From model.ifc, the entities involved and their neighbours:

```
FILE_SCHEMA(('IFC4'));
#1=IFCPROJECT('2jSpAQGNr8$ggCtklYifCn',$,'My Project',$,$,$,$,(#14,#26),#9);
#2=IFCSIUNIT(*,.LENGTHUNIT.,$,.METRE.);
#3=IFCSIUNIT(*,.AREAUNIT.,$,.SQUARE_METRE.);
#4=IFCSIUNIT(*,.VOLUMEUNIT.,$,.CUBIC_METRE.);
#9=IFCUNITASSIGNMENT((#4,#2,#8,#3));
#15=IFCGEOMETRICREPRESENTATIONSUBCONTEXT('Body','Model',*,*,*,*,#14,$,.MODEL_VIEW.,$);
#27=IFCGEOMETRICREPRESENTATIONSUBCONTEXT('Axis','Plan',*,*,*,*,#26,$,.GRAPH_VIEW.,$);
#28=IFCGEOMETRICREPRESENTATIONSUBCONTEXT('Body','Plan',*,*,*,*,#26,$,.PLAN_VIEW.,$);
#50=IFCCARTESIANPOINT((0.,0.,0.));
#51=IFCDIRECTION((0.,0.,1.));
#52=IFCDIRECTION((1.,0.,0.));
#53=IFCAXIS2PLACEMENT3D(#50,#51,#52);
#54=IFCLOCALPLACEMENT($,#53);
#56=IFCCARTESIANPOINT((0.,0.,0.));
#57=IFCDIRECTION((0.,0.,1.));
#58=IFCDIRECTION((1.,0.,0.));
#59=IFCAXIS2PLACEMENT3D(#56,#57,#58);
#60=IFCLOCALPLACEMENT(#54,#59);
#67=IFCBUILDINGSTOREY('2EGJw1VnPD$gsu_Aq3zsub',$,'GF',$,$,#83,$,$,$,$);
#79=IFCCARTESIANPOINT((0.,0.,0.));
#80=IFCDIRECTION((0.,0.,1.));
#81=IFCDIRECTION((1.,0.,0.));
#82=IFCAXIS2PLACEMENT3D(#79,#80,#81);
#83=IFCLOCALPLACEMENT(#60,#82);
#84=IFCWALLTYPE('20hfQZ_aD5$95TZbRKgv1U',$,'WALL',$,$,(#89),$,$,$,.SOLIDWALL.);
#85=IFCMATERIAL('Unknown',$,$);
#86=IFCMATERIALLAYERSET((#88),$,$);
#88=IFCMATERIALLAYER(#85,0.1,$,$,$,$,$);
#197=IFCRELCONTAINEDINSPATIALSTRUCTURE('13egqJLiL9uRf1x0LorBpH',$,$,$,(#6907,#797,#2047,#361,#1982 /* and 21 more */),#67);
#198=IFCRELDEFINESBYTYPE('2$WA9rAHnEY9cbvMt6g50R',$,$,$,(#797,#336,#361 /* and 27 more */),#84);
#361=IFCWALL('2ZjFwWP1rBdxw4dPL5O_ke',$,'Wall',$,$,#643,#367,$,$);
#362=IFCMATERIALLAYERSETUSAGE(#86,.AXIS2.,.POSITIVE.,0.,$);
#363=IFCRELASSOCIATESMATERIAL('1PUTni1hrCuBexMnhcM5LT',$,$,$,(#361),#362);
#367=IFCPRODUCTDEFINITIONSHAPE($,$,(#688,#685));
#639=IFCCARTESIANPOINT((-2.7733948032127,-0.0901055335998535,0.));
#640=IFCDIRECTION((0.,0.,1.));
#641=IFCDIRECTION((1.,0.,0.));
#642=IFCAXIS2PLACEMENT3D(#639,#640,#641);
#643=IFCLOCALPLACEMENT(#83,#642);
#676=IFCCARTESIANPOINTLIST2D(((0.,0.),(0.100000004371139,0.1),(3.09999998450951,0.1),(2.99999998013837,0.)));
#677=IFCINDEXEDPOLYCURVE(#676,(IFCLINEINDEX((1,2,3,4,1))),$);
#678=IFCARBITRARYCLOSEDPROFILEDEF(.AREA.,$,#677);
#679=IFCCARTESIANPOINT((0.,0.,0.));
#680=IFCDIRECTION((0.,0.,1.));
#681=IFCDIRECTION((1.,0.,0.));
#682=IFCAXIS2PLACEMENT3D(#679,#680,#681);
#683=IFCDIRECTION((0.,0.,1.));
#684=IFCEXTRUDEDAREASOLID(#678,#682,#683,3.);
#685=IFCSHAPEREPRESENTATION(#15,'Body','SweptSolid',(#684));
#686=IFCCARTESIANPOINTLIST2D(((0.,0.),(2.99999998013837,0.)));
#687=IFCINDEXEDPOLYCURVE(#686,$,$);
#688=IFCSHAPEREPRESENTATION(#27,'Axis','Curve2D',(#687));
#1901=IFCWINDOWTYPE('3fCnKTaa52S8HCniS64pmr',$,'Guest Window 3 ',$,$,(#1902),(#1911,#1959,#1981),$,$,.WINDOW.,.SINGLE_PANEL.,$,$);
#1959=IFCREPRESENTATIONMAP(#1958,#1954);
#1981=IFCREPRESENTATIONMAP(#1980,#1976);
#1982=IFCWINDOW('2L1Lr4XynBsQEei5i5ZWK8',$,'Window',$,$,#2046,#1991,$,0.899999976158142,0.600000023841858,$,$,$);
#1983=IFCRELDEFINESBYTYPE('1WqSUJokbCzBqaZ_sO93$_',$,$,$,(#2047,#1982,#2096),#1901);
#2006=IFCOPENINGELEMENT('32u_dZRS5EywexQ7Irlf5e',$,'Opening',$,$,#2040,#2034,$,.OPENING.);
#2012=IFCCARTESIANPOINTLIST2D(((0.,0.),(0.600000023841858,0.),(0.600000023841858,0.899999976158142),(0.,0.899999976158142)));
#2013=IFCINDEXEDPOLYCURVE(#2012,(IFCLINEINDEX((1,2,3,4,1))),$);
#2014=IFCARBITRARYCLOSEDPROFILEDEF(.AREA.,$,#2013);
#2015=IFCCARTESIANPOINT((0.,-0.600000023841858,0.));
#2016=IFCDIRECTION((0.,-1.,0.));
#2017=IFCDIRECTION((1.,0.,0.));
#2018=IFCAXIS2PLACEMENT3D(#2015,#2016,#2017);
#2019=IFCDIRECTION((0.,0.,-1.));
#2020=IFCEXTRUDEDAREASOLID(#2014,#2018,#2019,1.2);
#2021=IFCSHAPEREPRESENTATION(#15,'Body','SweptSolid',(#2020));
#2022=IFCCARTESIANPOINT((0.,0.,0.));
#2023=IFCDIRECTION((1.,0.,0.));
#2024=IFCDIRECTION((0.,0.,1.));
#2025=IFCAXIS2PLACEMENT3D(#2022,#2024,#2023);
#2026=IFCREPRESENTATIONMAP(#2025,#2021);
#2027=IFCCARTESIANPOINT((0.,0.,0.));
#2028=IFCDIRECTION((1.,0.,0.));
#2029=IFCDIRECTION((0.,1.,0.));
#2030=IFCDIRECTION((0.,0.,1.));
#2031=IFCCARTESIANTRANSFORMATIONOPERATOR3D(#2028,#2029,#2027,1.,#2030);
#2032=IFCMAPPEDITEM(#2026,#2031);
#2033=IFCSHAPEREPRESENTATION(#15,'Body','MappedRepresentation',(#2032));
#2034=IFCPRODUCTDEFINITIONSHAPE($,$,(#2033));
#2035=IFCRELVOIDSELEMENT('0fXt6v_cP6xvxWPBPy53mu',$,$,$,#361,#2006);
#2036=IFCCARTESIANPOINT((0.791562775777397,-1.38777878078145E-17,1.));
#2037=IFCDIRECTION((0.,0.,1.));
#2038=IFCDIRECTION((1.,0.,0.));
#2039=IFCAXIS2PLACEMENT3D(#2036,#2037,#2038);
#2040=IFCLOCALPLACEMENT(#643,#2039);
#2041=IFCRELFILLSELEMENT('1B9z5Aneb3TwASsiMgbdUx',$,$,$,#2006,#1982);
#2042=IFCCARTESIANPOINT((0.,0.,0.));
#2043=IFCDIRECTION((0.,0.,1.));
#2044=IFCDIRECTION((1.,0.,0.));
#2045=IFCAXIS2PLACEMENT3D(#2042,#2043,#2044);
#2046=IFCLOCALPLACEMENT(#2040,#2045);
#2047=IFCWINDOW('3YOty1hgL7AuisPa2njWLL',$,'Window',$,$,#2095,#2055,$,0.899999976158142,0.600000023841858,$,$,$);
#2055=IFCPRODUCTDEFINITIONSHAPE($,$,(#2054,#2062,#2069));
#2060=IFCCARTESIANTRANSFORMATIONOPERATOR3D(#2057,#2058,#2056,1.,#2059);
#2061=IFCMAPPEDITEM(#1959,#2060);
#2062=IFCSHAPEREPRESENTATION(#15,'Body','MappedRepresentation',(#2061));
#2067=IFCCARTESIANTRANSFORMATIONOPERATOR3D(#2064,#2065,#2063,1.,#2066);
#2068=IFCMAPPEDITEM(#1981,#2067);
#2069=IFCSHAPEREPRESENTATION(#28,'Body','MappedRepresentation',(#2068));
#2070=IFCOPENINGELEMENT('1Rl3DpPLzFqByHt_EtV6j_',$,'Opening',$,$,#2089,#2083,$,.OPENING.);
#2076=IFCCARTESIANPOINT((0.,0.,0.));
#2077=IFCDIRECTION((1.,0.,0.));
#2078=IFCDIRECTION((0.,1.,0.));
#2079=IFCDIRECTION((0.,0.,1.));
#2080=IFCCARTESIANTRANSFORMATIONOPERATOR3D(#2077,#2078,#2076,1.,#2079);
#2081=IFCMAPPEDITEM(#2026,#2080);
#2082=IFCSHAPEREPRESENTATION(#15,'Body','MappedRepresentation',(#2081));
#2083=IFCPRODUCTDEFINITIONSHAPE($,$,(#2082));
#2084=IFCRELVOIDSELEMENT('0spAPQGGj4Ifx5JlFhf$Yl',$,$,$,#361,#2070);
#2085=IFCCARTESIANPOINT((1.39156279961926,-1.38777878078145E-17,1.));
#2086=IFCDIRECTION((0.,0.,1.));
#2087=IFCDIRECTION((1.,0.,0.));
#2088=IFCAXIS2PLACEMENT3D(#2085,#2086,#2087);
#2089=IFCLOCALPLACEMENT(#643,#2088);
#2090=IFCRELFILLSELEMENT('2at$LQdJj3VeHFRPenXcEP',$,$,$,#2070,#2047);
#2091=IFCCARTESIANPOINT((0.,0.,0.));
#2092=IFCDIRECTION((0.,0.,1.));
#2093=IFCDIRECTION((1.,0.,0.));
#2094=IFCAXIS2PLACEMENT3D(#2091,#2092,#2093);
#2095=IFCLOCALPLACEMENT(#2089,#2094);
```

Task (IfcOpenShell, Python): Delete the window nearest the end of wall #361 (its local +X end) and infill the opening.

```python
import ifcopenshell
import ifcopenshell.api.feature
import ifcopenshell.api.root
import ifcopenshell.geom
import ifcopenshell.util.shape

model = ifcopenshell.open("model.ifc")
settings = ifcopenshell.geom.settings()


def volume(element):
    """Net volume in cubic metres, openings subtracted."""
    shape = ifcopenshell.geom.create_shape(settings, element)
    return ifcopenshell.util.shape.get_volume(shape.geometry)


window = model.by_guid("3YOty1hgL7AuisPa2njWLL")
opening = window.FillsVoids[0].RelatingOpeningElement
wall = opening.VoidsElements[0].RelatingBuildingElement
before = volume(wall)

ifcopenshell.api.root.remove_product(model, product=window)
ifcopenshell.api.feature.remove_feature(model, feature=opening)

after = volume(wall)

print(f"wall volume {before:.3f} -> {after:.3f} m3")

model.write("model-out.ifc")
```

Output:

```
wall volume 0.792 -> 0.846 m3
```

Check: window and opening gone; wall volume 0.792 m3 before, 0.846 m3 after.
